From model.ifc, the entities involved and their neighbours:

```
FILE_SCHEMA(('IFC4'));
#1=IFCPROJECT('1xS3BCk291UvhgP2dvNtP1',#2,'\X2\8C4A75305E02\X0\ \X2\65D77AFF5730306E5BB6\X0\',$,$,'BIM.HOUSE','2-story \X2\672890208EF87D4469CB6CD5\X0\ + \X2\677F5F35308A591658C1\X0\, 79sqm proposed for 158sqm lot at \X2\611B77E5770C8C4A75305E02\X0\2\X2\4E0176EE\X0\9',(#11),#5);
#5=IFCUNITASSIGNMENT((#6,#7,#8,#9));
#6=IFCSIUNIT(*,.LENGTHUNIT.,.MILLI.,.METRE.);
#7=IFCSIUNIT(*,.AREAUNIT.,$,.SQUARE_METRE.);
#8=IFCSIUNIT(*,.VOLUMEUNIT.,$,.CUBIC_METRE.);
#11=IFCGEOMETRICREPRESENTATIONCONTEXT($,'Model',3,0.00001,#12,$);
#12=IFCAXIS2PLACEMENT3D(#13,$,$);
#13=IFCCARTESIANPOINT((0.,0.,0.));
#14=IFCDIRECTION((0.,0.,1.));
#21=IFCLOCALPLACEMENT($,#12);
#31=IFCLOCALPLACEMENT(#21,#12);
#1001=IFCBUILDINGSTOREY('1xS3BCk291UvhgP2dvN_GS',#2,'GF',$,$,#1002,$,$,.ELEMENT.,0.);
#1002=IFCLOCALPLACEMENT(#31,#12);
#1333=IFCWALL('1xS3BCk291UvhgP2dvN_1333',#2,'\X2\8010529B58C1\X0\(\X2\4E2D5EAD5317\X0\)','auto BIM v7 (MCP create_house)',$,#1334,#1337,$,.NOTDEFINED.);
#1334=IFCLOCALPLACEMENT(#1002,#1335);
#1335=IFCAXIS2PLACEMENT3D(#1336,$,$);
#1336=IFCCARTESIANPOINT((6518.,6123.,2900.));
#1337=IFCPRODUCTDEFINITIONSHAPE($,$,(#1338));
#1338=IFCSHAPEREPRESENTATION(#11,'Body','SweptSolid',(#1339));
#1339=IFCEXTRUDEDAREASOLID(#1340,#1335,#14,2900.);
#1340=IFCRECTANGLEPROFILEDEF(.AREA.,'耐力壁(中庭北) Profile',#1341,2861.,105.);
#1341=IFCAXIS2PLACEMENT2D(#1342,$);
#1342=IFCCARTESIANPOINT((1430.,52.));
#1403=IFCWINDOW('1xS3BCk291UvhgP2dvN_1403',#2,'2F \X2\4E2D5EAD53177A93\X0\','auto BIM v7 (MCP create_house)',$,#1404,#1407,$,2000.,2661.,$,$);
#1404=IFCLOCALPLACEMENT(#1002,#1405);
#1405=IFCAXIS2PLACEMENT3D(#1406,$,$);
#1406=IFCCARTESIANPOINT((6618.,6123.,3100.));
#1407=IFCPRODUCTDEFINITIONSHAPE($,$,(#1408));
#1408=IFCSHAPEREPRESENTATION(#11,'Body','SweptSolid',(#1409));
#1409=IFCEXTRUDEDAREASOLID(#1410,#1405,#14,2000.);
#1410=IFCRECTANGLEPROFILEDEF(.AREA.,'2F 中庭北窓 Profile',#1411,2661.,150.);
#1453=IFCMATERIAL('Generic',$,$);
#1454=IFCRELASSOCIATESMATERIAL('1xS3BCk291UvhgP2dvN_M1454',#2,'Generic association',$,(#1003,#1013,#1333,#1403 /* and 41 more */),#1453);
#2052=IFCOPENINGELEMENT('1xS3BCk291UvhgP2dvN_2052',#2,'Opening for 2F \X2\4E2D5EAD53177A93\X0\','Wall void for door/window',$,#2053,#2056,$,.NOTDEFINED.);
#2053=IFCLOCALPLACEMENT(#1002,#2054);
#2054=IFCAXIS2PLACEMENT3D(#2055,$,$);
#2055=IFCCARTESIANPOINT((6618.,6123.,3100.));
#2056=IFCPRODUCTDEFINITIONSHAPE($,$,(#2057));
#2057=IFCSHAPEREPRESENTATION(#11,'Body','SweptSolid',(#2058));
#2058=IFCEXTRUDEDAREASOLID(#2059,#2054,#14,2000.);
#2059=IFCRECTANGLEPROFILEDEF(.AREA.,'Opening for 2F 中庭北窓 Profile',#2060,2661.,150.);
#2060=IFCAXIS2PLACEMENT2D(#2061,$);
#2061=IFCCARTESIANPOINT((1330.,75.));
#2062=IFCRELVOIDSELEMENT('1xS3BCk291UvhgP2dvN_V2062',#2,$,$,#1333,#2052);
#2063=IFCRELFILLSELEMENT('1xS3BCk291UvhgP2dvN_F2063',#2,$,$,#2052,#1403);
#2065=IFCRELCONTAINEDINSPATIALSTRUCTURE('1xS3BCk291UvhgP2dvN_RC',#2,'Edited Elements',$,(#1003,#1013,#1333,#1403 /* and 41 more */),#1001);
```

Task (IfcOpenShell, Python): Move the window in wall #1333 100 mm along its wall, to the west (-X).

```python
import ifcopenshell
import ifcopenshell.api.geometry
import ifcopenshell.util.placement

model = ifcopenshell.open("model.ifc")

window = model.by_guid("1xS3BCk291UvhgP2dvN_1403")
opening = window.FillsVoids[0].RelatingOpeningElement
wall = opening.VoidsElements[0].RelatingBuildingElement

wall_matrix = ifcopenshell.util.placement.get_local_placement(wall.ObjectPlacement)
shift = wall_matrix[:3, 0] * -100.0
before = ifcopenshell.util.placement.get_local_placement(window.ObjectPlacement)[:3, 3].copy()

# The window is not placed relative to its opening, so move both.
for product in (opening, window):
    matrix = ifcopenshell.util.placement.get_local_placement(product.ObjectPlacement)
    matrix[:3, 3] += shift
    ifcopenshell.api.geometry.edit_object_placement(model, product=product, matrix=matrix, is_si=False)

after = ifcopenshell.util.placement.get_local_placement(window.ObjectPlacement)[:3, 3]
print("window moved by", (after - before).round(3) + 0.0)

model.write("model_updated.ifc")
```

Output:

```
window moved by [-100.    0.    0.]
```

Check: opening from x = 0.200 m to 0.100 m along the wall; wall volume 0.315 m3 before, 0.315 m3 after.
